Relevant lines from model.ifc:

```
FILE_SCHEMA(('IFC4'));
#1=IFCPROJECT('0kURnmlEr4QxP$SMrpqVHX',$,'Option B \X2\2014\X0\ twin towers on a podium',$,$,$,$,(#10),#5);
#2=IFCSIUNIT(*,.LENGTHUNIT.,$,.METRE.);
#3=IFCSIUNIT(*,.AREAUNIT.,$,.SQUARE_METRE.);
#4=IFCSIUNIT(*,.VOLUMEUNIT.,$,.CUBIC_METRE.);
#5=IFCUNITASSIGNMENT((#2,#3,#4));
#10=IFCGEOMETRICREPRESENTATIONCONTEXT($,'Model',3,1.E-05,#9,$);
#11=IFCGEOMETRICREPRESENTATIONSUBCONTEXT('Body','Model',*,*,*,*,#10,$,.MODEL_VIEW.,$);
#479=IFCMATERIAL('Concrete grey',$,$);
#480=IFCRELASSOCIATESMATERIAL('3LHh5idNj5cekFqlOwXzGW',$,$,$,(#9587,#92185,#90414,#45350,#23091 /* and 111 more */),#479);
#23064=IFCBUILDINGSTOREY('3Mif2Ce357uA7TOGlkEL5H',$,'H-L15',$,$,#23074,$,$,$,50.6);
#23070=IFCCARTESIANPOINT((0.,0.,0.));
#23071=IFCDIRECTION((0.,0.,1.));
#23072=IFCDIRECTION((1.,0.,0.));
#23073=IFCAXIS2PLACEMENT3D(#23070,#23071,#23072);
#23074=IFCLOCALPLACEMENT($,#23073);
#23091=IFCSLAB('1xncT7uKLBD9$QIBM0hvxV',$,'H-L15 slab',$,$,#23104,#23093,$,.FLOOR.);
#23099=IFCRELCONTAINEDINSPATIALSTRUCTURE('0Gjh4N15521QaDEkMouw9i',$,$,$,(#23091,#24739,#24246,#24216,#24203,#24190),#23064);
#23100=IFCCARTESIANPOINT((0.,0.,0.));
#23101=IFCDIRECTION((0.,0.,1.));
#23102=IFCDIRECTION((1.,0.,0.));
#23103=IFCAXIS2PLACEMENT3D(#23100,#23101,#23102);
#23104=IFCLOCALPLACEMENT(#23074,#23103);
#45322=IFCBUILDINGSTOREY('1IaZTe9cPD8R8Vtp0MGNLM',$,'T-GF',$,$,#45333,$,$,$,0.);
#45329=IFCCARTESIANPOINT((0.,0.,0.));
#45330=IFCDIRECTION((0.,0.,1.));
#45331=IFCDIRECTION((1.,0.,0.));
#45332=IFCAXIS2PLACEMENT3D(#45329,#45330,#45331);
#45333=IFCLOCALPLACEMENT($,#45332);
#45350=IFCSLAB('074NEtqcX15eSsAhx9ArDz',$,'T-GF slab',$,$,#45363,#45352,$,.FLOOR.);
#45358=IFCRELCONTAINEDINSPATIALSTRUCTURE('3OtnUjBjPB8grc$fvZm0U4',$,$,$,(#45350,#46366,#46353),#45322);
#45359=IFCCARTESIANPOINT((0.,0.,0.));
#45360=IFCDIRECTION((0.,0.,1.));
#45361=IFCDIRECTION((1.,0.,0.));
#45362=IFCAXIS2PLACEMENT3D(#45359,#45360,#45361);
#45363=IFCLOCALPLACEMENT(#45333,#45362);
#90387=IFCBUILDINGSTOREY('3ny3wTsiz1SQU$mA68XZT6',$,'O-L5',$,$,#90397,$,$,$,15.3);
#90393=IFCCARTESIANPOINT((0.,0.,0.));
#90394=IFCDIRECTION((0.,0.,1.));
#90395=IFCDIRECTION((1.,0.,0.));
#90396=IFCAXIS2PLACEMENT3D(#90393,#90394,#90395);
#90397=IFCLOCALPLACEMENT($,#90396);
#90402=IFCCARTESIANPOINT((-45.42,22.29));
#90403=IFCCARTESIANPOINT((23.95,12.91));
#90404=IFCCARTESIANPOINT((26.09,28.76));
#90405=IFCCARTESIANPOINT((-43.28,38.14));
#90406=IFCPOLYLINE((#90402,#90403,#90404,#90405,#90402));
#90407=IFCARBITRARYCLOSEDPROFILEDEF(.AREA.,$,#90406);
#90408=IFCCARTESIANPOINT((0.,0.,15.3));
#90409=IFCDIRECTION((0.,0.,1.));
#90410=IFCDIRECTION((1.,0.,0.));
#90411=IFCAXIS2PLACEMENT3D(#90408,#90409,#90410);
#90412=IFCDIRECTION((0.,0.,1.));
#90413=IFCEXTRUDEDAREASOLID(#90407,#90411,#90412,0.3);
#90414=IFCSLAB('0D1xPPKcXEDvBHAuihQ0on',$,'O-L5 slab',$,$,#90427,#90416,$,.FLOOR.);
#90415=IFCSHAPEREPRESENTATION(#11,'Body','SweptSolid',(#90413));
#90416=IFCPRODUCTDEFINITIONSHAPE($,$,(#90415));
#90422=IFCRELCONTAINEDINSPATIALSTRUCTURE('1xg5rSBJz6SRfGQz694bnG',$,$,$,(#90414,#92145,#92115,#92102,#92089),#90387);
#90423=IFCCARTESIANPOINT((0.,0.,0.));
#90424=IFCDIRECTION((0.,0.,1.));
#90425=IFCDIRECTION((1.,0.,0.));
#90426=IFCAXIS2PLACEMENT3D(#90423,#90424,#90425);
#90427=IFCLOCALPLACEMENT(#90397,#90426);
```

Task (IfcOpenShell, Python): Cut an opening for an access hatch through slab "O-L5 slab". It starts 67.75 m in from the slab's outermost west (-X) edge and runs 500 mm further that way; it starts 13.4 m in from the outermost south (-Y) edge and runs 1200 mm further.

```python
import numpy as np
import ifcopenshell
import ifcopenshell.api.feature
import ifcopenshell.api.geometry
import ifcopenshell.api.root
import ifcopenshell.geom
import ifcopenshell.util.placement
import ifcopenshell.util.representation
import ifcopenshell.util.shape
import ifcopenshell.util.unit

model = ifcopenshell.open("model.ifc")
unit_scale = ifcopenshell.util.unit.calculate_unit_scale(model)
settings = ifcopenshell.geom.settings()


def volume(element):
    """Net volume in cubic metres, openings subtracted."""
    shape = ifcopenshell.geom.create_shape(settings, element)
    return ifcopenshell.util.shape.get_volume(shape.geometry)


slab = model.by_guid("0D1xPPKcXEDvBHAuihQ0on")
before = volume(slab)

# Extent in the slab's own axes, in metres. The edges named are its -X and -Y sides.
slab_shape = ifcopenshell.geom.create_shape(settings, slab)
vertices = ifcopenshell.util.shape.get_vertices(slab_shape.geometry)
x_min, y_min, bottom = vertices.min(axis=0)
top = vertices[:, 2].max()

opening = ifcopenshell.api.root.create_entity(model, ifc_class="IfcOpeningElement", name="Access hatch opening", predefined_type="OPENING")
context = ifcopenshell.util.representation.get_context(model, "Model", "Body", "MODEL_VIEW")
width, depth = 0.5, 1.2
outline = [(0.0, 0.0), (width, 0.0), (width, depth), (0.0, depth), (0.0, 0.0)]
# Overshoot both faces by 50 mm so the cut is clean.
shape = ifcopenshell.api.geometry.add_slab_representation(
    model, context=context, depth=top - bottom + 0.1, polyline=outline
)
ifcopenshell.api.geometry.assign_representation(model, product=opening, representation=shape)

matrix = ifcopenshell.util.placement.get_local_placement(slab.ObjectPlacement)
matrix[:, 3] = matrix @ np.append(np.array([x_min + 67.75, y_min + 13.4, bottom - 0.05]) / unit_scale, 1.0)
ifcopenshell.api.geometry.edit_object_placement(model, product=opening, matrix=matrix, is_si=False)
ifcopenshell.api.feature.add_feature(model, feature=opening, element=slab)

after = volume(slab)

print(f"slab volume {before:.3f} -> {after:.3f} m3")

model.write("model_updated.ifc")
```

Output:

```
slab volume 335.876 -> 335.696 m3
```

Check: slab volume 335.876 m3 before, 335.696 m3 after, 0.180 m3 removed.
